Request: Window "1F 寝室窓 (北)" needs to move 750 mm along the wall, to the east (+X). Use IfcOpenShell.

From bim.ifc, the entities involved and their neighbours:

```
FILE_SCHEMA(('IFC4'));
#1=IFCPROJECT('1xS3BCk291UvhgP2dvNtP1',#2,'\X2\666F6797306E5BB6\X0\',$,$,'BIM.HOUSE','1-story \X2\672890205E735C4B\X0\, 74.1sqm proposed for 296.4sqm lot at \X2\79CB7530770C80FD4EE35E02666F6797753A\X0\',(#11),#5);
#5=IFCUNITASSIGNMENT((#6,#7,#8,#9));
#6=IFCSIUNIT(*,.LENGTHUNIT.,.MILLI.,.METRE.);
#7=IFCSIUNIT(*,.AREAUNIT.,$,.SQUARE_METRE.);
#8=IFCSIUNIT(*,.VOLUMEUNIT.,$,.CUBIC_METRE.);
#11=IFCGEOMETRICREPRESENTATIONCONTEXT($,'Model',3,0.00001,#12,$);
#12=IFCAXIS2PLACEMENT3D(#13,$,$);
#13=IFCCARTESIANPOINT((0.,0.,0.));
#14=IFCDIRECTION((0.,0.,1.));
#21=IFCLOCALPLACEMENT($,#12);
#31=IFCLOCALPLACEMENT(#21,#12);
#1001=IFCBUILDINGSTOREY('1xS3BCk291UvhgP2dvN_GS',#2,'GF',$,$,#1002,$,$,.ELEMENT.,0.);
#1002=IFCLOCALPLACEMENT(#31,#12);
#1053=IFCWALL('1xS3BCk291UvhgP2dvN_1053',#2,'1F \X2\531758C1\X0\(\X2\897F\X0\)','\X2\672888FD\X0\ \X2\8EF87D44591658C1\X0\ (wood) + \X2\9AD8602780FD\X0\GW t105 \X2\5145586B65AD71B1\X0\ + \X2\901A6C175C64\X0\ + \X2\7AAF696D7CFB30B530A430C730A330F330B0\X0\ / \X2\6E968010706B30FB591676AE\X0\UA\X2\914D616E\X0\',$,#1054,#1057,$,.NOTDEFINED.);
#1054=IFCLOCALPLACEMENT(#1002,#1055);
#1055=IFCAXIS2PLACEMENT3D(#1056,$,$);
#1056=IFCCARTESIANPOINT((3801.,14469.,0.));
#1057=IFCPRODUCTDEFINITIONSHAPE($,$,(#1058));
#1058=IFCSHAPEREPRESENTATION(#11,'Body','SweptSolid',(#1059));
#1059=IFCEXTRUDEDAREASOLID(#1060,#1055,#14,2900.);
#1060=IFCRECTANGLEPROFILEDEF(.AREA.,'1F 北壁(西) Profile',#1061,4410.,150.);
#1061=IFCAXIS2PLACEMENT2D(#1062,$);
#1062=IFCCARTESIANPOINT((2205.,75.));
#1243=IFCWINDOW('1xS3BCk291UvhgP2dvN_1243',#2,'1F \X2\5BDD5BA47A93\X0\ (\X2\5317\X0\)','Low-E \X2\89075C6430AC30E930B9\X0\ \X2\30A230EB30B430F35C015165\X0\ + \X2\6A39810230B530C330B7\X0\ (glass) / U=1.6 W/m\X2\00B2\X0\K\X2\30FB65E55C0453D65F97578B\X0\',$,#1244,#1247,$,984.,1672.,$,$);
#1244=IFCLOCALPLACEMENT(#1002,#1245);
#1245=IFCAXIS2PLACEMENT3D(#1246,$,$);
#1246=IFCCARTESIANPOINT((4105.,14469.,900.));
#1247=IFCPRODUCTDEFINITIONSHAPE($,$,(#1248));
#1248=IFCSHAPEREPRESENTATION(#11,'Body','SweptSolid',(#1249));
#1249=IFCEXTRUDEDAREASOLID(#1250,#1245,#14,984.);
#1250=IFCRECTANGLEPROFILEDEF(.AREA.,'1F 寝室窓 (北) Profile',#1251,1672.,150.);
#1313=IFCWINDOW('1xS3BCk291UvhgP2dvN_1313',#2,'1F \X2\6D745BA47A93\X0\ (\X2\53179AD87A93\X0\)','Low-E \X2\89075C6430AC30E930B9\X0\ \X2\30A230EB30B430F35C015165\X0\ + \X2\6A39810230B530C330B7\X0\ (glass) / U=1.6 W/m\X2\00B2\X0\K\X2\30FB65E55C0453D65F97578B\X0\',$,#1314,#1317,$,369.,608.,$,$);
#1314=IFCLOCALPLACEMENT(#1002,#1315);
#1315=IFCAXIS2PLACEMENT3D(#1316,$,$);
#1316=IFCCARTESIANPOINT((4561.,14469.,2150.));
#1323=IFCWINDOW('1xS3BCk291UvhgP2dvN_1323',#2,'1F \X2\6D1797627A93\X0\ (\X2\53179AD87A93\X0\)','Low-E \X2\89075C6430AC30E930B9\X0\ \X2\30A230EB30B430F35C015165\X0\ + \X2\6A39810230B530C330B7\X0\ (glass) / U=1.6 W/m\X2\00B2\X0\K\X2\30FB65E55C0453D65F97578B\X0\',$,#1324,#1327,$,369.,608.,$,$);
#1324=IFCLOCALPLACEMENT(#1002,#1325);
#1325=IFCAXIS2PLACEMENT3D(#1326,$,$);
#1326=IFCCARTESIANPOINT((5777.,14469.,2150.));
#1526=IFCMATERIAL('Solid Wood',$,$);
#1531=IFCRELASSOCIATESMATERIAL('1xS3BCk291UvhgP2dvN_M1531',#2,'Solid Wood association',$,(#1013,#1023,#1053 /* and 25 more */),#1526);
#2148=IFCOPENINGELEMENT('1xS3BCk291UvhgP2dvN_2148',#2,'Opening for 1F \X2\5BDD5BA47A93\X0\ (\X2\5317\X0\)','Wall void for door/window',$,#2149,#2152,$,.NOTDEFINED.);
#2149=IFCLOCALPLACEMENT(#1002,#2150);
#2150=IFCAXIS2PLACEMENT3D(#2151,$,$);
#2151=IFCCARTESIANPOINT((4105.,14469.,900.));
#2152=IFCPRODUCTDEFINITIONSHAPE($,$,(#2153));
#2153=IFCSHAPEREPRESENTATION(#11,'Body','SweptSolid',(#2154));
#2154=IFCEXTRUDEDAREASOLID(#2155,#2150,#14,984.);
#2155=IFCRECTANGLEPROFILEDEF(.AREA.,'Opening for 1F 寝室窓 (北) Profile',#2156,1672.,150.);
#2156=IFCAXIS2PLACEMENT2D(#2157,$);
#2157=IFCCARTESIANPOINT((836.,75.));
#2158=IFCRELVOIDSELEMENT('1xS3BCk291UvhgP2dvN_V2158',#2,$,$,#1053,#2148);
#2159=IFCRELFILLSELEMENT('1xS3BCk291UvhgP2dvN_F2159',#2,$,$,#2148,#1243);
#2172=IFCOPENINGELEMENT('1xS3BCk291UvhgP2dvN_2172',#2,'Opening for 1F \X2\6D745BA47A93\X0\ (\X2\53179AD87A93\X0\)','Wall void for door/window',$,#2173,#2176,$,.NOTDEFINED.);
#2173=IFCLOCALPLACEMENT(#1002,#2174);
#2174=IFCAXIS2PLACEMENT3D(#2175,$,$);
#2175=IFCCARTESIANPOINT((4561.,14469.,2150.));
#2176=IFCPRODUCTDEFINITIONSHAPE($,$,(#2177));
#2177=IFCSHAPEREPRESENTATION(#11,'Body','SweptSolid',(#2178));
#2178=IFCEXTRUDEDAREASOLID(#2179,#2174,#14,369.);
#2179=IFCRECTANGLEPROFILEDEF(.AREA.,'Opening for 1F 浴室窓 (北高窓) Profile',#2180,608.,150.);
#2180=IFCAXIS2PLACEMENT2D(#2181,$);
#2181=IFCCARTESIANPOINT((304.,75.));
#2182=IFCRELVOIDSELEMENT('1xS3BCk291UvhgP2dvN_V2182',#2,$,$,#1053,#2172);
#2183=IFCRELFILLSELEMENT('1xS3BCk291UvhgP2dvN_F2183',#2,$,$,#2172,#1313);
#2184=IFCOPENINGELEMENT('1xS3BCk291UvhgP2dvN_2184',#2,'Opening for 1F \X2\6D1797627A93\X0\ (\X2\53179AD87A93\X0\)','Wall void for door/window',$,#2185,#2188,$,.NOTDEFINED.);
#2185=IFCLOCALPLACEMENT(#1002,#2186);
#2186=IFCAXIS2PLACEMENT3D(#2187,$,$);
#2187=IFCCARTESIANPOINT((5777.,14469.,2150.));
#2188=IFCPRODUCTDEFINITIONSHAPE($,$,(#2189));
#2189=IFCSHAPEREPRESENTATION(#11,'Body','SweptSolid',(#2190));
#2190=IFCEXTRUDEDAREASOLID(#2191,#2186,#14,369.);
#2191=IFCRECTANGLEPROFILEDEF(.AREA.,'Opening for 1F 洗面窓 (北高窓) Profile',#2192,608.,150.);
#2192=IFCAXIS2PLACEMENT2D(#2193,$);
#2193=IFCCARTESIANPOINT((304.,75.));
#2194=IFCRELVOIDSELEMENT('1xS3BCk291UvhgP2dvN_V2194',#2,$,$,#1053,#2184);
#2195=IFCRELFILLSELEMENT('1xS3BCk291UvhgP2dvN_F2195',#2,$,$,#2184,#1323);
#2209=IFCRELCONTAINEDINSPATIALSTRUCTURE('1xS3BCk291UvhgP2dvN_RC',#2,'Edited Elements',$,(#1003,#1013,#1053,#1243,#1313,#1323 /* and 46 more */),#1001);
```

```python
import ifcopenshell
import ifcopenshell.api.geometry
import ifcopenshell.util.placement
import ifcopenshell.util.unit

model = ifcopenshell.open("bim.ifc")
unit_scale = ifcopenshell.util.unit.calculate_unit_scale(model)

window = model.by_guid("1xS3BCk291UvhgP2dvN_1243")
opening = window.FillsVoids[0].RelatingOpeningElement
wall = opening.VoidsElements[0].RelatingBuildingElement

wall_matrix = ifcopenshell.util.placement.get_local_placement(wall.ObjectPlacement)
shift = wall_matrix[:3, 0] * 0.75 / unit_scale
before = ifcopenshell.util.placement.get_local_placement(window.ObjectPlacement)[:3, 3].copy()

# The window is not placed relative to its opening, so move both.
for product in (opening, window):
    matrix = ifcopenshell.util.placement.get_local_placement(product.ObjectPlacement)
    matrix[:3, 3] += shift
    ifcopenshell.api.geometry.edit_object_placement(model, product=product, matrix=matrix, is_si=False)

after = ifcopenshell.util.placement.get_local_placement(window.ObjectPlacement)[:3, 3]
print("window moved by", (after - before).round(3) + 0.0)

model.write("bim_rev.ifc")
```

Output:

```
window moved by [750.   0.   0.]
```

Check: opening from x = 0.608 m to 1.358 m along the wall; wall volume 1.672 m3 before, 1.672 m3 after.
